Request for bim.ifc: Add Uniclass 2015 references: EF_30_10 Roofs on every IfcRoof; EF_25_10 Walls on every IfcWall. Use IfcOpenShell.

First a look at what the model holds.

```python
import ifcopenshell

model = ifcopenshell.open("bim.ifc")
print(model.schema)
print("classifications:", [c.Name for c in model.by_type("IfcClassification")])
for ifc_class in ("IfcDoor", "IfcRoof", "IfcStair", "IfcWall", "IfcWindow"):
    print(ifc_class, len(model.by_type(ifc_class)))
```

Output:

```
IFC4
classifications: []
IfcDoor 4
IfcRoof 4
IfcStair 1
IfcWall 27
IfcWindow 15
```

```python
import ifcopenshell
import ifcopenshell.api.classification

model = ifcopenshell.open("bim.ifc")

system = ifcopenshell.api.classification.add_classification(model, classification="Uniclass 2015")

codes = {
    "IfcRoof": ("EF_30_10", "Roofs"),
    "IfcWall": ("EF_25_10", "Walls"),
}
for ifc_class, (code, name) in codes.items():
    products = model.by_type(ifc_class)
    ifcopenshell.api.classification.add_reference(
        model, products=products, classification=system, identification=code, name=name
    )
    print(code, len(products))

model.write("bim_updated.ifc")
```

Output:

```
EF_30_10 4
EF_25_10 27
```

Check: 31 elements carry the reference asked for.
